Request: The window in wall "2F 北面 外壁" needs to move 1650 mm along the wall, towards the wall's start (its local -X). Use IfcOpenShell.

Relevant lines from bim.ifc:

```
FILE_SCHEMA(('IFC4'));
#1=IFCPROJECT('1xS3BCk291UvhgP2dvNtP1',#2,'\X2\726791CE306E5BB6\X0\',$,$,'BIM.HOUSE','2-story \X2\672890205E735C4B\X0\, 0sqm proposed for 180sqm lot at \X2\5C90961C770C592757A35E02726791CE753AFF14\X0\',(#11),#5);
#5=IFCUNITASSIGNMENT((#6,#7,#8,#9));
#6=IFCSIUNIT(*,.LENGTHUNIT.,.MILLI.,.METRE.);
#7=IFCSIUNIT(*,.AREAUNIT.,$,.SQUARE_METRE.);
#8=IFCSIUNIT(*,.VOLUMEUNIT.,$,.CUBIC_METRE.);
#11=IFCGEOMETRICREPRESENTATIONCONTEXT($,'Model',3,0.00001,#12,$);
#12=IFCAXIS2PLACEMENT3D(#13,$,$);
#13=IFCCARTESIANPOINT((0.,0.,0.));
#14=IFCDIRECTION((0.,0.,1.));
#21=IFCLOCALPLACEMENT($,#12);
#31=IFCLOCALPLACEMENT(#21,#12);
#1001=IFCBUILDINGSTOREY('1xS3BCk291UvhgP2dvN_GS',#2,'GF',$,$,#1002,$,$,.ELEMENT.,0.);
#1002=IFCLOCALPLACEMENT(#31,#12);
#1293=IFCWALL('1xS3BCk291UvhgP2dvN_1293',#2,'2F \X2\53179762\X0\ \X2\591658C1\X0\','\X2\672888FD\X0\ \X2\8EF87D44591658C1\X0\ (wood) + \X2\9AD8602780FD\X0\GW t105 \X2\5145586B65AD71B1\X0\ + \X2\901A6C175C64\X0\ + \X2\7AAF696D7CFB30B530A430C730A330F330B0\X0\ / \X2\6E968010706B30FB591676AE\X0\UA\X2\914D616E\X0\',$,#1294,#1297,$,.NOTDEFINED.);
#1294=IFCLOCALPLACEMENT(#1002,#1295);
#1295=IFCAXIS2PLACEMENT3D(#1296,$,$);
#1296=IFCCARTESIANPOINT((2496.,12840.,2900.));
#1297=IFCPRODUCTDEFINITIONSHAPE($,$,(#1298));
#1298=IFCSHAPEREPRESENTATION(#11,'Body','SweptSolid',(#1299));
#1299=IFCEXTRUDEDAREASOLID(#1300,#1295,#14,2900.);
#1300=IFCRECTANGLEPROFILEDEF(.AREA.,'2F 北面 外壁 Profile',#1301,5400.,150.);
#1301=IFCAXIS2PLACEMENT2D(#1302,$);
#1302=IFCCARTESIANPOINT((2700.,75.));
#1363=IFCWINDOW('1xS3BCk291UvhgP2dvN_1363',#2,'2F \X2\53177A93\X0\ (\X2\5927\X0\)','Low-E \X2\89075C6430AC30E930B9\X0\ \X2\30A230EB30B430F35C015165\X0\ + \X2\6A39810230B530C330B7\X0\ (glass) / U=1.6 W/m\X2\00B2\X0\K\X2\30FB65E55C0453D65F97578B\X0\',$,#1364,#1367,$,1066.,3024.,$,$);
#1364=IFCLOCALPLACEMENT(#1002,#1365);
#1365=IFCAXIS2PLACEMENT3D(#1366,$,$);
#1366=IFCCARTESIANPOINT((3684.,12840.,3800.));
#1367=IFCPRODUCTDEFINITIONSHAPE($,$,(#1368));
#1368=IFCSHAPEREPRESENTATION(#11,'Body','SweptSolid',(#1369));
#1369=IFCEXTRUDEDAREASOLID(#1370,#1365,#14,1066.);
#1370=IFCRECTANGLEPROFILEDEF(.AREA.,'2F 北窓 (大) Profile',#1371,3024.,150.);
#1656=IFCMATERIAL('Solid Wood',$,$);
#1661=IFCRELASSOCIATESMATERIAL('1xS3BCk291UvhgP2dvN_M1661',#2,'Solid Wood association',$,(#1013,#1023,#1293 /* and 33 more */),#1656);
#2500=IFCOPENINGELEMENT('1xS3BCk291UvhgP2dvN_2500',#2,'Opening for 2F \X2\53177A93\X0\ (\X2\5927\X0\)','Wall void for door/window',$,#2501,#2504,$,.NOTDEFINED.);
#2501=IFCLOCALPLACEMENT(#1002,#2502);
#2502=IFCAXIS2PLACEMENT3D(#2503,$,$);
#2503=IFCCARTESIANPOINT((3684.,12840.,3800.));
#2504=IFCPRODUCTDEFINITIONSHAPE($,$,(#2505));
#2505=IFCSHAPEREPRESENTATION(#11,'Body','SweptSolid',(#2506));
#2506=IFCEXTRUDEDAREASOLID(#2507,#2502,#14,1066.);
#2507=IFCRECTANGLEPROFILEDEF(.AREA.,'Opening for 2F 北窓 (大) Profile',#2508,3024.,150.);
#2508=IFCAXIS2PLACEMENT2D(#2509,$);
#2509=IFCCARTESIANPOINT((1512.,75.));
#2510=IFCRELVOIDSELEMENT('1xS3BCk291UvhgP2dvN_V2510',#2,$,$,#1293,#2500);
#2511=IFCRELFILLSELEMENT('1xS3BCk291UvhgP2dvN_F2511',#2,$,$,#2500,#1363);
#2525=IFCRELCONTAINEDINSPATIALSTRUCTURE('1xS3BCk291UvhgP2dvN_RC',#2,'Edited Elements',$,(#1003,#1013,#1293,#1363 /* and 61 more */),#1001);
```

```python
import ifcopenshell
import ifcopenshell.api.geometry
import ifcopenshell.util.placement

model = ifcopenshell.open("bim.ifc")

window = model.by_id(1363)
opening = window.FillsVoids[0].RelatingOpeningElement
wall = opening.VoidsElements[0].RelatingBuildingElement

wall_matrix = ifcopenshell.util.placement.get_local_placement(wall.ObjectPlacement)
shift = wall_matrix[:3, 0] * -1650.0
before = ifcopenshell.util.placement.get_local_placement(window.ObjectPlacement)[:3, 3].copy()

# The window is not placed relative to its opening, so move both.
for product in (opening, window):
    matrix = ifcopenshell.util.placement.get_local_placement(product.ObjectPlacement)
    matrix[:3, 3] += shift
    ifcopenshell.api.geometry.edit_object_placement(model, product=product, matrix=matrix, is_si=False)

after = ifcopenshell.util.placement.get_local_placement(window.ObjectPlacement)[:3, 3]
print("window moved by", (after - before).round(3) + 0.0)

model.write("bim-out.ifc")
```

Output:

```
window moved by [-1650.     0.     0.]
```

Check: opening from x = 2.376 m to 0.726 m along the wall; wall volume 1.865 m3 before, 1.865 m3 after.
